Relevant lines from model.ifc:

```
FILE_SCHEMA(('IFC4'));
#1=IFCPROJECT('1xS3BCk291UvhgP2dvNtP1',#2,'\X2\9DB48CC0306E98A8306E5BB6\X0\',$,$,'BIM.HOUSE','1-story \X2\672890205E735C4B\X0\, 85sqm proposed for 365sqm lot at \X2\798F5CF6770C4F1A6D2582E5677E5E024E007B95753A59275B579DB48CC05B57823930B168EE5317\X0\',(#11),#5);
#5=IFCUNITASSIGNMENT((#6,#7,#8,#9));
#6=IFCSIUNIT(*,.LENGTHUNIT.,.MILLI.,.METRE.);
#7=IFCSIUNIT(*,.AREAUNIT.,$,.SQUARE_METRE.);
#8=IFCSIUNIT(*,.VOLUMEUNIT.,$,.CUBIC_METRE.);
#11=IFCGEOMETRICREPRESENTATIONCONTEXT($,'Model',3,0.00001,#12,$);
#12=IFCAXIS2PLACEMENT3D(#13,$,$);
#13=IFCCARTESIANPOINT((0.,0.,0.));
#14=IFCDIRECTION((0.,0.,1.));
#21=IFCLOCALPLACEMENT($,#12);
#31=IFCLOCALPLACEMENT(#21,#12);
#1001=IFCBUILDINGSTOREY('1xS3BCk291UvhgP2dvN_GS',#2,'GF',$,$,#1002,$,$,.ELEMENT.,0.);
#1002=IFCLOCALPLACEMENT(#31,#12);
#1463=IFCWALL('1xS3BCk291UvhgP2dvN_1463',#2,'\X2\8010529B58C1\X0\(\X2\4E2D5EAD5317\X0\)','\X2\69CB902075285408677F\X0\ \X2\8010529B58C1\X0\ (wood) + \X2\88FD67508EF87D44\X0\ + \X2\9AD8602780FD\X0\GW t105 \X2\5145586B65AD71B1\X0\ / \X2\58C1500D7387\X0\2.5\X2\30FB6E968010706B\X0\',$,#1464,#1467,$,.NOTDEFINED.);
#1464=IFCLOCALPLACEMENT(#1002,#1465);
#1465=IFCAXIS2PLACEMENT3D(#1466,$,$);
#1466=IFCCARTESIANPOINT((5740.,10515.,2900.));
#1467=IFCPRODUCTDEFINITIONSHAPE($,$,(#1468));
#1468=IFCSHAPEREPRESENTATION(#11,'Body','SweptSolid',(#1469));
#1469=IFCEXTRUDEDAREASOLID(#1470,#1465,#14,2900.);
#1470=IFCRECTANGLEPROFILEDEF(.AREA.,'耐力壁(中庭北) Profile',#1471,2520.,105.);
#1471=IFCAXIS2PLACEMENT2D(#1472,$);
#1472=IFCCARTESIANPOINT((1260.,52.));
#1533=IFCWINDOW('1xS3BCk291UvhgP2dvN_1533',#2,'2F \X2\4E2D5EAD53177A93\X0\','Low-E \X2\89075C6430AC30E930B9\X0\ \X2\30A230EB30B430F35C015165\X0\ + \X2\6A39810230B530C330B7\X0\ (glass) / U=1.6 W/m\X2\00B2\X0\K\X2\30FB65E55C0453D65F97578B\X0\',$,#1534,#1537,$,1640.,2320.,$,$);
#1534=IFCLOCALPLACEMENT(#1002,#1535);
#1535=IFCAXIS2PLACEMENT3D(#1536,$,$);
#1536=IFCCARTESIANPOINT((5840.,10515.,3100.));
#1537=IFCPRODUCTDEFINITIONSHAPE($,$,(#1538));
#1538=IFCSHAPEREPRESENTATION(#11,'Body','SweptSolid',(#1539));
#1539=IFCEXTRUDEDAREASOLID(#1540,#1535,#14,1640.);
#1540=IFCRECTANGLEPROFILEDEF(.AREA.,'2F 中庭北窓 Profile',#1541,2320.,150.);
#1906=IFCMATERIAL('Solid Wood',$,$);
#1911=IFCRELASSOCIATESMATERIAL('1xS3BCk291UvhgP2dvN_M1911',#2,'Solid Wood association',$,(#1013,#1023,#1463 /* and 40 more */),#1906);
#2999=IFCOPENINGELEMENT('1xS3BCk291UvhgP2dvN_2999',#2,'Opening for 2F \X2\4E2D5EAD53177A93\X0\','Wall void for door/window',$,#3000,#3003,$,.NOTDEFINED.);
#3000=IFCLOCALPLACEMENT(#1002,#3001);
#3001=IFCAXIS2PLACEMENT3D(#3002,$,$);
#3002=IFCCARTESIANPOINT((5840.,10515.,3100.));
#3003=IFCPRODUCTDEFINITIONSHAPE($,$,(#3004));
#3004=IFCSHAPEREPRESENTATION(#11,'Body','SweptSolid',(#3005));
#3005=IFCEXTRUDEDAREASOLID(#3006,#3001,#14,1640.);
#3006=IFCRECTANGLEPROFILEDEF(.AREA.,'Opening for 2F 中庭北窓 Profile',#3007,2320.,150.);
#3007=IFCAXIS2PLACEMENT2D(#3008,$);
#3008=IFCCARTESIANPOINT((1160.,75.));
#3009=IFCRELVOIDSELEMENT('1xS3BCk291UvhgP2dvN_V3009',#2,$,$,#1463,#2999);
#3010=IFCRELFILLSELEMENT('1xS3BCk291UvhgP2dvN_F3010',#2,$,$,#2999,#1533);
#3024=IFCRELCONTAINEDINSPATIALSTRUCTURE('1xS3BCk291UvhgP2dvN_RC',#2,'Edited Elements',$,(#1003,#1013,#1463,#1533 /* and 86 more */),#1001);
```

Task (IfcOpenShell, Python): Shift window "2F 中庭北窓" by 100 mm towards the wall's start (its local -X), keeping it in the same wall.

```python
import ifcopenshell
import ifcopenshell.api.geometry
import ifcopenshell.util.placement
import ifcopenshell.util.unit

model = ifcopenshell.open("model.ifc")
unit_scale = ifcopenshell.util.unit.calculate_unit_scale(model)

window = model.by_id(1533)
opening = window.FillsVoids[0].RelatingOpeningElement
wall = opening.VoidsElements[0].RelatingBuildingElement

wall_matrix = ifcopenshell.util.placement.get_local_placement(wall.ObjectPlacement)
shift = wall_matrix[:3, 0] * -0.1 / unit_scale
before = ifcopenshell.util.placement.get_local_placement(window.ObjectPlacement)[:3, 3].copy()

# The window is not placed relative to its opening, so move both.
for product in (opening, window):
    matrix = ifcopenshell.util.placement.get_local_placement(product.ObjectPlacement)
    matrix[:3, 3] += shift
    ifcopenshell.api.geometry.edit_object_placement(model, product=product, matrix=matrix, is_si=False)

after = ifcopenshell.util.placement.get_local_placement(window.ObjectPlacement)[:3, 3]
print("window moved by", (after - before).round(3) + 0.0)

model.write("model-out.ifc")
```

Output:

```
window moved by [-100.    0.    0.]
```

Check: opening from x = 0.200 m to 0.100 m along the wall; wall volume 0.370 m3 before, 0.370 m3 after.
